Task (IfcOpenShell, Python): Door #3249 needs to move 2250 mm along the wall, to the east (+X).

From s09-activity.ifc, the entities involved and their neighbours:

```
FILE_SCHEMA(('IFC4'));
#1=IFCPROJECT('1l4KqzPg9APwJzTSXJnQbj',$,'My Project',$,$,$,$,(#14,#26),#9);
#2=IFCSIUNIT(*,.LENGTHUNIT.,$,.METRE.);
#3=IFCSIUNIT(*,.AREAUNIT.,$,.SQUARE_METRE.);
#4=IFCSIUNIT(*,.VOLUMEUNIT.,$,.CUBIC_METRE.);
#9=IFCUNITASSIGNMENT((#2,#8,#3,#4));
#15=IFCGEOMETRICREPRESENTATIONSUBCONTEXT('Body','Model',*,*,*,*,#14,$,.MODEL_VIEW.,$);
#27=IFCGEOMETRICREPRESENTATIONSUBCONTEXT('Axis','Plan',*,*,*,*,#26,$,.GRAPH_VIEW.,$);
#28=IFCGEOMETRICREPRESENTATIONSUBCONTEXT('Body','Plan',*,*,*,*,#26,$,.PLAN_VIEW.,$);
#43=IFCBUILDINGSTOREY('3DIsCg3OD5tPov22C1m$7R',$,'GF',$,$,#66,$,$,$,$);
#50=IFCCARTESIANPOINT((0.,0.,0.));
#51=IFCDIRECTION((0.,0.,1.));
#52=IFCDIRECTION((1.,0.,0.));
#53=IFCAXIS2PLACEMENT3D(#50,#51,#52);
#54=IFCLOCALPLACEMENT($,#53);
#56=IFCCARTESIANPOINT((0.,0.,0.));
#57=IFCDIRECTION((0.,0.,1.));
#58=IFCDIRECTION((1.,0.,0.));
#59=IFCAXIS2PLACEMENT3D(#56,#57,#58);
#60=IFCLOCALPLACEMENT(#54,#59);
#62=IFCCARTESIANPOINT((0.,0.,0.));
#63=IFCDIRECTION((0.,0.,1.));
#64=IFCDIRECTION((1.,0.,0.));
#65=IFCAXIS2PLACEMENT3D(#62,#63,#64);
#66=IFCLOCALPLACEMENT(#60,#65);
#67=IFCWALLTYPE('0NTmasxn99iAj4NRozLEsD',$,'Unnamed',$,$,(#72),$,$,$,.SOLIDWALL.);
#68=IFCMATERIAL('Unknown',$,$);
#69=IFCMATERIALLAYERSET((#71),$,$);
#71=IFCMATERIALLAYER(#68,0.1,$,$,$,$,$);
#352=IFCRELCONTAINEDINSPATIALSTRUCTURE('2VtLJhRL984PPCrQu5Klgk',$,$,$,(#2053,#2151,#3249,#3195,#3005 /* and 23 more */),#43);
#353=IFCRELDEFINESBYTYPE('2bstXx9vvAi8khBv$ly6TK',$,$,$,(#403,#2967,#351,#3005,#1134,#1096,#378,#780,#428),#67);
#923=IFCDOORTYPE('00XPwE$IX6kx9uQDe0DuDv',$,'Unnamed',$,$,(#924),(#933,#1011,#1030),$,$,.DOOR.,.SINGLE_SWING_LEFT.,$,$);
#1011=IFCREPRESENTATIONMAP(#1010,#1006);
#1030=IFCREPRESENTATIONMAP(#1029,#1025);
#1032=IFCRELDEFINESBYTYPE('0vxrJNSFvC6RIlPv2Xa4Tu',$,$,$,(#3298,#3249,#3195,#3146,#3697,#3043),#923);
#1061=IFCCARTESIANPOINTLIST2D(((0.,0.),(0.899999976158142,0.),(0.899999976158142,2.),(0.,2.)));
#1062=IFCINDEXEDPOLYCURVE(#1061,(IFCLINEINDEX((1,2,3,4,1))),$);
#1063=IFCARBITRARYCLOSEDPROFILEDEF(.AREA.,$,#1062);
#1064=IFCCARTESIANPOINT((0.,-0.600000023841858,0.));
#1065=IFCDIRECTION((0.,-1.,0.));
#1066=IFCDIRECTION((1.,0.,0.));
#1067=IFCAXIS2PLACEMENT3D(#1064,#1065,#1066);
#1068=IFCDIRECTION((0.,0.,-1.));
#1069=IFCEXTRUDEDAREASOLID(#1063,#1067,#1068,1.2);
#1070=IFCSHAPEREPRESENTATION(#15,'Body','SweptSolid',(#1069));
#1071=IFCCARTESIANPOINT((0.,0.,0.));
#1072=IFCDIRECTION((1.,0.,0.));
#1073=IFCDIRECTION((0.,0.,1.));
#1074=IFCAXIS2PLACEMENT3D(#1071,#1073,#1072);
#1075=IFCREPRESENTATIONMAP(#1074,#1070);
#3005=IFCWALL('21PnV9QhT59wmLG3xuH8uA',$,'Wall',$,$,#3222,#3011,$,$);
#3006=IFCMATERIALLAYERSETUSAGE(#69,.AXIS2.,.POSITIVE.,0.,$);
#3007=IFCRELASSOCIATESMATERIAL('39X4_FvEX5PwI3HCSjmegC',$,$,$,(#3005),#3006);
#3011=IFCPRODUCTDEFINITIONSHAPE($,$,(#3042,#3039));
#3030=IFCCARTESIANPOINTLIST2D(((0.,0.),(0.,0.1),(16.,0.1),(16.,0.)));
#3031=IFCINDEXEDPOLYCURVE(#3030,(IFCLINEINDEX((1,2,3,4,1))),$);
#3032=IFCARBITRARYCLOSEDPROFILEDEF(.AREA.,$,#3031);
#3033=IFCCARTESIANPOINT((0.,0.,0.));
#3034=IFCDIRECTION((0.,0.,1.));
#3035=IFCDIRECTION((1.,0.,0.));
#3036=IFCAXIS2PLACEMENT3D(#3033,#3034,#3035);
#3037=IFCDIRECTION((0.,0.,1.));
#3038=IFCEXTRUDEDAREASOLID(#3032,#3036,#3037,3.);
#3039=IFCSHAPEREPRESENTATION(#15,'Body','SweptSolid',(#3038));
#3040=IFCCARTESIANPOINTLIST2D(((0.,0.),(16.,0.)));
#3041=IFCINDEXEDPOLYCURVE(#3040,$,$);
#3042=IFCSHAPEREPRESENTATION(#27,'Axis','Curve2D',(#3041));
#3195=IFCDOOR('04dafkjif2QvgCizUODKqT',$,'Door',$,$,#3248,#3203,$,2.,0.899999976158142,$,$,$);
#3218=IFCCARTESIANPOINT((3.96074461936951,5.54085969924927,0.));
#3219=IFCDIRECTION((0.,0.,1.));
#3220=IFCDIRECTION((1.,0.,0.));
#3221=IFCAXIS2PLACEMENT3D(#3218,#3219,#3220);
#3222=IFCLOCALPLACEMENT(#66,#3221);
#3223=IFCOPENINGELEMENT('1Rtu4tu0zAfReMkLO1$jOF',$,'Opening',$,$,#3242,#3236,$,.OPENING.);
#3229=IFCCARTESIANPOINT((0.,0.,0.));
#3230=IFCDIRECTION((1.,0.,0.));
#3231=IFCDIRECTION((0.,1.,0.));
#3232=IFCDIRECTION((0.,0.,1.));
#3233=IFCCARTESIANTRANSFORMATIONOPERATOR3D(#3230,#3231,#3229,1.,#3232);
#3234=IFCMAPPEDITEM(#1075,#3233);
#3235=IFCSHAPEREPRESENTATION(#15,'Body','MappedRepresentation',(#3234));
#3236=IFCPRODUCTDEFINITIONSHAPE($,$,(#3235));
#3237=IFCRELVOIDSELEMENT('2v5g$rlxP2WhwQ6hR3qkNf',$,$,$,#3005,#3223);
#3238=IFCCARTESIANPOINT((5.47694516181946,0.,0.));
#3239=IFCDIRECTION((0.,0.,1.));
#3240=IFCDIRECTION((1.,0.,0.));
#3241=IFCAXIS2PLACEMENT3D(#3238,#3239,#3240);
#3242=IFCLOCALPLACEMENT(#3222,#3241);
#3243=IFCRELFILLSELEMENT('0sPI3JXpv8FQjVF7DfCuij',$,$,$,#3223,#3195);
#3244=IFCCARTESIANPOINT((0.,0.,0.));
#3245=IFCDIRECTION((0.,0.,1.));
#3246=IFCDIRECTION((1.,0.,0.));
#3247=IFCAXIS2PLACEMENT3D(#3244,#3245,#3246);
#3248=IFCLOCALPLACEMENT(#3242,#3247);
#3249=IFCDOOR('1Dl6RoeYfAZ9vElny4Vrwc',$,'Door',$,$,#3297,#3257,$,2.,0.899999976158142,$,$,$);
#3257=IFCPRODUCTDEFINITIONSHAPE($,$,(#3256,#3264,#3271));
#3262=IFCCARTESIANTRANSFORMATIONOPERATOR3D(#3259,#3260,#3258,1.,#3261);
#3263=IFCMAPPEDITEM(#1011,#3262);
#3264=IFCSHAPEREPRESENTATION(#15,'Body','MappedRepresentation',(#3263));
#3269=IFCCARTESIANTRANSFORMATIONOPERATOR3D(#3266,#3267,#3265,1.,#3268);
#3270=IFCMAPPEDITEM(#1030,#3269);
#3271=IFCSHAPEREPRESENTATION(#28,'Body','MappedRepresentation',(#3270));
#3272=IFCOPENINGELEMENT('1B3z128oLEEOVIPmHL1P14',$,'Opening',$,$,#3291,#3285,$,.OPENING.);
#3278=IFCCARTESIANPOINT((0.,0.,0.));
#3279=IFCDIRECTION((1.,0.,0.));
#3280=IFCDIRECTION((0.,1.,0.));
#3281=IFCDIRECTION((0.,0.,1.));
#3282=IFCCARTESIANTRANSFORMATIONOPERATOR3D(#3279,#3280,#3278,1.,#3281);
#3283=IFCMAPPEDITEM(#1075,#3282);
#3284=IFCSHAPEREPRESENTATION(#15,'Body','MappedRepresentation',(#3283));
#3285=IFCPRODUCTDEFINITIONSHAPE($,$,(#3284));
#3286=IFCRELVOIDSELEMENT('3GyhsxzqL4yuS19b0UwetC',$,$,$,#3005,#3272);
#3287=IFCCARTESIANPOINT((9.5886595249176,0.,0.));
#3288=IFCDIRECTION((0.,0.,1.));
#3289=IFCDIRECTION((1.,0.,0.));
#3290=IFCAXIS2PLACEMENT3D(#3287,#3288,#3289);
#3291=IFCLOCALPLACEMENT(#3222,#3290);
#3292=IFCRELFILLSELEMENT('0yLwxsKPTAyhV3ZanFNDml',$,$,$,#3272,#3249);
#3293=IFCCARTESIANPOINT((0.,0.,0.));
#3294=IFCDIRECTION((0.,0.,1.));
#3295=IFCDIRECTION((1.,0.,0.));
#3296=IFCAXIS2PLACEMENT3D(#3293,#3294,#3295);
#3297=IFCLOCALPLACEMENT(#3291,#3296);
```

```python
import ifcopenshell
import ifcopenshell.api.geometry
import ifcopenshell.util.placement

model = ifcopenshell.open("s09-activity.ifc")

door = model.by_guid("1Dl6RoeYfAZ9vElny4Vrwc")
opening = door.FillsVoids[0].RelatingOpeningElement
wall = opening.VoidsElements[0].RelatingBuildingElement

wall_matrix = ifcopenshell.util.placement.get_local_placement(wall.ObjectPlacement)
shift = wall_matrix[:3, 0] * 2.25
before = ifcopenshell.util.placement.get_local_placement(door.ObjectPlacement)[:3, 3].copy()

# The door is placed relative to its opening, so it follows when the opening moves.
matrix = ifcopenshell.util.placement.get_local_placement(opening.ObjectPlacement)
matrix[:3, 3] += shift
ifcopenshell.api.geometry.edit_object_placement(
    model, product=opening, matrix=matrix, is_si=False, should_transform_children=True
)

after = ifcopenshell.util.placement.get_local_placement(door.ObjectPlacement)[:3, 3]
print("door moved by", (after - before).round(3) + 0.0)

model.write("s09-activity_edited.ifc")
```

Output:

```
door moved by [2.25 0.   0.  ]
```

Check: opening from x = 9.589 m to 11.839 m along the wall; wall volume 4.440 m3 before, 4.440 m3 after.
